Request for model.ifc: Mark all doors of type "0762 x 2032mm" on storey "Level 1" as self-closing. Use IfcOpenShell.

First a look at what the model holds.

```python
import ifcopenshell
import ifcopenshell.util.element

model = ifcopenshell.open("model.ifc")
print(model.schema)
storey = next(s for s in model.by_type("IfcBuildingStorey") if s.Name == "Level 1")
doors = [e for e in ifcopenshell.util.element.get_decomposition(storey) if e.is_a("IfcDoor")]
seen = {}
for e in doors:
    element_type = ifcopenshell.util.element.get_type(e)
    key = (element_type.Name if element_type != e and element_type else None, ifcopenshell.util.element.get_pset(e, "Pset_DoorCommon", "SelfClosing"))
    seen[key] = seen.get(key, 0) + 1
for (name, value), count in sorted(seen.items(), key=str):
    print(count, "x", name, "|", value)
```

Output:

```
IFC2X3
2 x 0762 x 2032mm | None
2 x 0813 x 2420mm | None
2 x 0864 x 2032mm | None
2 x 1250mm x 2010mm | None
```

```python
import ifcopenshell
import ifcopenshell.api.pset
import ifcopenshell.util.element

model = ifcopenshell.open("model.ifc")

storey = next(s for s in model.by_type("IfcBuildingStorey") if s.Name == "Level 1")
doors = [e for e in ifcopenshell.util.element.get_decomposition(storey) if e.is_a("IfcDoor")]

count = 0
for e in doors:
    element_type = ifcopenshell.util.element.get_type(e)
    if element_type in (None, e) or element_type.Name != "0762 x 2032mm":
        continue
    # add_pset returns the element's existing set when there is one.
    pset = ifcopenshell.api.pset.add_pset(model, product=e, name="Pset_DoorCommon")
    ifcopenshell.api.pset.edit_pset(model, pset=pset, properties={"SelfClosing": True})
    count += 1

print(count, "doors updated")

model.write("model_rev.ifc")
```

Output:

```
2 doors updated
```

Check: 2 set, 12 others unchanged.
